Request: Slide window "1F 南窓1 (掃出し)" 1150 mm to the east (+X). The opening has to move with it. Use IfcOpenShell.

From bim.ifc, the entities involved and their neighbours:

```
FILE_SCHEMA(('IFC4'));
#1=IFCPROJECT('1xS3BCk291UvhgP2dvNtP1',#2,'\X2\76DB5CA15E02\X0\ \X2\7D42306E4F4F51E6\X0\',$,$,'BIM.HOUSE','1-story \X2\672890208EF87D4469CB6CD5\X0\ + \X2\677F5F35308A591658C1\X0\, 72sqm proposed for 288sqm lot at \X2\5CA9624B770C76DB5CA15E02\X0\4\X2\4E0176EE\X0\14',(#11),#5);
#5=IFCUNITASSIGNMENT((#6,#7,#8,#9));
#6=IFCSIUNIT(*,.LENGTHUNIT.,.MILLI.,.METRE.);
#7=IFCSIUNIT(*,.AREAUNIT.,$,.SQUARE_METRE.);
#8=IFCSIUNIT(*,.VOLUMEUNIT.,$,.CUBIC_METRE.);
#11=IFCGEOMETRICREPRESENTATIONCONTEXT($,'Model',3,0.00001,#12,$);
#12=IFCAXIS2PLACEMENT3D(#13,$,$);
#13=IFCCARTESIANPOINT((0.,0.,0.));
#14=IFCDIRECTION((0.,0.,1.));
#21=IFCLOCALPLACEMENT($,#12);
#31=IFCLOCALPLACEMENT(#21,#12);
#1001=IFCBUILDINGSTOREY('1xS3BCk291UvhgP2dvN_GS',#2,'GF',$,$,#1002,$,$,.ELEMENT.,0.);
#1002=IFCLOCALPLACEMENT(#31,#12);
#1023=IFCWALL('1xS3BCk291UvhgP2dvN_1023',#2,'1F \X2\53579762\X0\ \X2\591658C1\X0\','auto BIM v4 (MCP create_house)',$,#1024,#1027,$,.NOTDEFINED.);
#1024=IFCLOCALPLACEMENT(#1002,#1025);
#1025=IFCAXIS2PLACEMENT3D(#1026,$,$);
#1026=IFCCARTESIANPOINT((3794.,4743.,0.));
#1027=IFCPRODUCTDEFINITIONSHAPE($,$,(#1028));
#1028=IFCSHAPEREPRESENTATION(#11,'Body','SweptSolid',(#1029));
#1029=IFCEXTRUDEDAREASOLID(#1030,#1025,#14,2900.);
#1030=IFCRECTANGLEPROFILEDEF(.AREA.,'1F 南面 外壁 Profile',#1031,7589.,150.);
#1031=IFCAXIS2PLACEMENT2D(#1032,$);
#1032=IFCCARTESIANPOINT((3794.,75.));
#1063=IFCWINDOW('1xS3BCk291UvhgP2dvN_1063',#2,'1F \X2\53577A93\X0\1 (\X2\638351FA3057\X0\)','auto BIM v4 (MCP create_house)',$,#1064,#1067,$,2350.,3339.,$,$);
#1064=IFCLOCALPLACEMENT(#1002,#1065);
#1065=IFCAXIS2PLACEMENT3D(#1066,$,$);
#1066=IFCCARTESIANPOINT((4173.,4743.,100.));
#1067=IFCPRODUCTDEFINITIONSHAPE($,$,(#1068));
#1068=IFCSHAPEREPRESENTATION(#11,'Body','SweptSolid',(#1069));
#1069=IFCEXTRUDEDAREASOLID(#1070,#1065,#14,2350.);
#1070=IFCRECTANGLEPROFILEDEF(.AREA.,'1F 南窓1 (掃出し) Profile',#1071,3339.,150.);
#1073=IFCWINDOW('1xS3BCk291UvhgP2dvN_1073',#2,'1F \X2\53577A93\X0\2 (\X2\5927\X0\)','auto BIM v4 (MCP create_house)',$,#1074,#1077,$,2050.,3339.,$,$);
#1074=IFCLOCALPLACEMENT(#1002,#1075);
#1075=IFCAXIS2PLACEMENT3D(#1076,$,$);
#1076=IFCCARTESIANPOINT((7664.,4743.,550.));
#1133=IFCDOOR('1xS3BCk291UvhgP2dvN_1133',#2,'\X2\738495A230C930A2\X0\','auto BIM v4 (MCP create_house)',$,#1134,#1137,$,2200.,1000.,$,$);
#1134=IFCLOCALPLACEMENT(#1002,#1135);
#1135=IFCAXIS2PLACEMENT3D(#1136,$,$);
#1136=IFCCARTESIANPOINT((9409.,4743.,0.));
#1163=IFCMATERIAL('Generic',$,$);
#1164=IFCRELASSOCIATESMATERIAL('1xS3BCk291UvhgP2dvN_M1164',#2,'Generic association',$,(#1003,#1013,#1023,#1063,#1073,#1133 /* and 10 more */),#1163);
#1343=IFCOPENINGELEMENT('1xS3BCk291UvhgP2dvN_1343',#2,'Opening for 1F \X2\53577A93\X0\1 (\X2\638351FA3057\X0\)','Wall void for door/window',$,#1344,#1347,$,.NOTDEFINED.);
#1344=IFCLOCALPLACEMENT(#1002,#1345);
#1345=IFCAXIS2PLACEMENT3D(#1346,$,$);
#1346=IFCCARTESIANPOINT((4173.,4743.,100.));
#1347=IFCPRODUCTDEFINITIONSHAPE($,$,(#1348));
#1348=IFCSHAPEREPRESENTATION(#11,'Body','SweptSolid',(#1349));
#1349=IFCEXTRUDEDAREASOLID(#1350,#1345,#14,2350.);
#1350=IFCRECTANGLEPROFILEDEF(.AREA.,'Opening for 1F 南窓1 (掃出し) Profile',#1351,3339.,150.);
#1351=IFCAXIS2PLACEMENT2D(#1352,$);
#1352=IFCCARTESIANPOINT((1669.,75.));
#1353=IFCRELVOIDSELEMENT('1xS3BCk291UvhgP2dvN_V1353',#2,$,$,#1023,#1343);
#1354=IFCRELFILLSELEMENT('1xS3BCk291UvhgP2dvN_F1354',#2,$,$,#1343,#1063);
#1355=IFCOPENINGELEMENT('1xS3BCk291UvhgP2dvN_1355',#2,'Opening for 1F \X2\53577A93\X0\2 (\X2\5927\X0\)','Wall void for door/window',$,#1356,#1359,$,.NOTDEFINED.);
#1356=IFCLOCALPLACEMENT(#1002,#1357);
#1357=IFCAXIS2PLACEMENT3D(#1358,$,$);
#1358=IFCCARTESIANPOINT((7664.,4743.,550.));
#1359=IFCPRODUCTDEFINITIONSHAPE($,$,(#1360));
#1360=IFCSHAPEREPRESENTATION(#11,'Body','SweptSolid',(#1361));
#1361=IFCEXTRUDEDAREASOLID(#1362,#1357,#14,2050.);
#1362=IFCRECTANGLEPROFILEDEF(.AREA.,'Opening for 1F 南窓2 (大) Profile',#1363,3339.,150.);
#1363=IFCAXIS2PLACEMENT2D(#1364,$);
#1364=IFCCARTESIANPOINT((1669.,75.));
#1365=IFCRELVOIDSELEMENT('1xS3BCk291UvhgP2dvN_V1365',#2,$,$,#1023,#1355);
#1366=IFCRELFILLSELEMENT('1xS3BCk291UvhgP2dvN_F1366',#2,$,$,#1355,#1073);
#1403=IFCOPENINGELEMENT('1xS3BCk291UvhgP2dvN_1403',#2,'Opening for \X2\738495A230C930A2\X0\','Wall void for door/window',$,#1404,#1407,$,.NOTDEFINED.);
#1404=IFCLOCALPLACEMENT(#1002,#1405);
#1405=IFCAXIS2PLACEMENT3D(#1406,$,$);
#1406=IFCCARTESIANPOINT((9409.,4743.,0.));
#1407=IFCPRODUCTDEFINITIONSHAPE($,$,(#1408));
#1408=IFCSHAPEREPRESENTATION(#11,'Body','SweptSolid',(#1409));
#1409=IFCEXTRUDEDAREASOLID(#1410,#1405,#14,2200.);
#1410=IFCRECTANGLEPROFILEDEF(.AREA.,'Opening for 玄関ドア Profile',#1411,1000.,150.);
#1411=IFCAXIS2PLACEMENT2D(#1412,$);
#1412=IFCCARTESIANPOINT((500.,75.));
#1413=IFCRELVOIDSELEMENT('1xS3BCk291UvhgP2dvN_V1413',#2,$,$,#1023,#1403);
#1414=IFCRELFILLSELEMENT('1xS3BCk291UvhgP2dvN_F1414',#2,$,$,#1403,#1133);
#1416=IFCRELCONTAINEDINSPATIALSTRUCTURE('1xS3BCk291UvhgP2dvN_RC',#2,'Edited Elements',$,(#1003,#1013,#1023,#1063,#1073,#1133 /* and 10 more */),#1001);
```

```python
import ifcopenshell
import ifcopenshell.api.geometry
import ifcopenshell.util.placement

model = ifcopenshell.open("bim.ifc")

window = model.by_guid("1xS3BCk291UvhgP2dvN_1063")
opening = window.FillsVoids[0].RelatingOpeningElement
wall = opening.VoidsElements[0].RelatingBuildingElement

wall_matrix = ifcopenshell.util.placement.get_local_placement(wall.ObjectPlacement)
shift = wall_matrix[:3, 0] * 1150.0
before = ifcopenshell.util.placement.get_local_placement(window.ObjectPlacement)[:3, 3].copy()

# The window is not placed relative to its opening, so move both.
for product in (opening, window):
    matrix = ifcopenshell.util.placement.get_local_placement(product.ObjectPlacement)
    matrix[:3, 3] += shift
    ifcopenshell.api.geometry.edit_object_placement(model, product=product, matrix=matrix, is_si=False)

after = ifcopenshell.util.placement.get_local_placement(window.ObjectPlacement)[:3, 3]
print("window moved by", (after - before).round(3) + 0.0)

model.write("bim-out.ifc")
```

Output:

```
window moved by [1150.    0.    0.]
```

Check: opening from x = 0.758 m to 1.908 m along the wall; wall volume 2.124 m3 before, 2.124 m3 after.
